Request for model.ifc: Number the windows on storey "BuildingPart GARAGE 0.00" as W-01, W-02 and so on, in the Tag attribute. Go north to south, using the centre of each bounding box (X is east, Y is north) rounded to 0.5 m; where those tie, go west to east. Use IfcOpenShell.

First a look at what the model holds.

```python
import ifcopenshell
import ifcopenshell.util.element
import ifcopenshell.util.placement

model = ifcopenshell.open("model.ifc")
print(model.schema)
storey = next(s for s in model.by_type("IfcBuildingStorey") if s.Name == "BuildingPart GARAGE 0.00")
windows = [e for e in ifcopenshell.util.element.get_decomposition(storey) if e.is_a("IfcWindow")]
for e in sorted(windows, key=lambda e: e.id()):
    origin = ifcopenshell.util.placement.get_local_placement(e.ObjectPlacement)[:3, 3]
    print(e.id(), e.Tag, e.Name, origin.round(2) + 0.0, sep=" | ")
```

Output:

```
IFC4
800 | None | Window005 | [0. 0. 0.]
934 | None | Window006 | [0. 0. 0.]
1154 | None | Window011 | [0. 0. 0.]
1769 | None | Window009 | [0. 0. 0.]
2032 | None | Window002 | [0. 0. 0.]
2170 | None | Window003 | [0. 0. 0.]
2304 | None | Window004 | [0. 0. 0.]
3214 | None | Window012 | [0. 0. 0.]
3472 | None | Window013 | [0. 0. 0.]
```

```python
import ifcopenshell
import ifcopenshell.geom
import ifcopenshell.util.element
import ifcopenshell.util.shape

model = ifcopenshell.open("model.ifc")
settings = ifcopenshell.geom.settings()
settings.set("use-world-coords", True)


def centre(element):
    shape = ifcopenshell.geom.create_shape(settings, element)
    return ifcopenshell.util.shape.get_bbox_centroid(shape.geometry)


storey = next(s for s in model.by_type("IfcBuildingStorey") if s.Name == "BuildingPart GARAGE 0.00")
windows = [e for e in ifcopenshell.util.element.get_decomposition(storey) if e.is_a("IfcWindow")]

# Insertion points can sit at a corner or the storey origin, so sort by the geometry (in metres).
centres = {e: centre(e) for e in windows}
windows.sort(key=lambda e: (-round(centres[e][1] / 0.5), centres[e][0]))

for i, e in enumerate(windows, start=1):
    number = f"W-{i:02d}"
    e.Tag = number
    print(e.id(), number)

model.write("model_updated.ifc")
```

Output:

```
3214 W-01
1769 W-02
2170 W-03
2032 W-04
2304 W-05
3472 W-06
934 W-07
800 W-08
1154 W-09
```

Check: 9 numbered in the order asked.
